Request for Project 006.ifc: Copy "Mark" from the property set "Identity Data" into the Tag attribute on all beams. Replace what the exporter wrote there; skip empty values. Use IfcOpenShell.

First a look at what the model holds.

```python
import ifcopenshell
import ifcopenshell.util.element

model = ifcopenshell.open("Project 006.ifc")
print(model.schema)
beams = model.by_type("IfcBeam")
print(len(beams), "beams")
for e in beams[:8]:
    source = ifcopenshell.util.element.get_pset(e, "Identity Data", "Mark")
    target = e.Tag
    print(e.id(), repr(source), repr(target), sep=" | ")
```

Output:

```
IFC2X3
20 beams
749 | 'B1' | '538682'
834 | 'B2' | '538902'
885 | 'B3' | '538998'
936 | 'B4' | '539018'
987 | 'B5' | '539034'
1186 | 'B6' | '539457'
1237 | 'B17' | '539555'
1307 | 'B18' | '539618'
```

```python
import ifcopenshell
import ifcopenshell.util.element

model = ifcopenshell.open("Project 006.ifc")

count = 0
for e in model.by_type("IfcBeam"):
    value = ifcopenshell.util.element.get_pset(e, "Identity Data", "Mark")
    current = e.Tag
    if not value or not value.strip() or current == value:
        continue
    e.Tag = value
    count += 1

print(count, "beams updated")

model.write("Project 006_v2.ifc")
```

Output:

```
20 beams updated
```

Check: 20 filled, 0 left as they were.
